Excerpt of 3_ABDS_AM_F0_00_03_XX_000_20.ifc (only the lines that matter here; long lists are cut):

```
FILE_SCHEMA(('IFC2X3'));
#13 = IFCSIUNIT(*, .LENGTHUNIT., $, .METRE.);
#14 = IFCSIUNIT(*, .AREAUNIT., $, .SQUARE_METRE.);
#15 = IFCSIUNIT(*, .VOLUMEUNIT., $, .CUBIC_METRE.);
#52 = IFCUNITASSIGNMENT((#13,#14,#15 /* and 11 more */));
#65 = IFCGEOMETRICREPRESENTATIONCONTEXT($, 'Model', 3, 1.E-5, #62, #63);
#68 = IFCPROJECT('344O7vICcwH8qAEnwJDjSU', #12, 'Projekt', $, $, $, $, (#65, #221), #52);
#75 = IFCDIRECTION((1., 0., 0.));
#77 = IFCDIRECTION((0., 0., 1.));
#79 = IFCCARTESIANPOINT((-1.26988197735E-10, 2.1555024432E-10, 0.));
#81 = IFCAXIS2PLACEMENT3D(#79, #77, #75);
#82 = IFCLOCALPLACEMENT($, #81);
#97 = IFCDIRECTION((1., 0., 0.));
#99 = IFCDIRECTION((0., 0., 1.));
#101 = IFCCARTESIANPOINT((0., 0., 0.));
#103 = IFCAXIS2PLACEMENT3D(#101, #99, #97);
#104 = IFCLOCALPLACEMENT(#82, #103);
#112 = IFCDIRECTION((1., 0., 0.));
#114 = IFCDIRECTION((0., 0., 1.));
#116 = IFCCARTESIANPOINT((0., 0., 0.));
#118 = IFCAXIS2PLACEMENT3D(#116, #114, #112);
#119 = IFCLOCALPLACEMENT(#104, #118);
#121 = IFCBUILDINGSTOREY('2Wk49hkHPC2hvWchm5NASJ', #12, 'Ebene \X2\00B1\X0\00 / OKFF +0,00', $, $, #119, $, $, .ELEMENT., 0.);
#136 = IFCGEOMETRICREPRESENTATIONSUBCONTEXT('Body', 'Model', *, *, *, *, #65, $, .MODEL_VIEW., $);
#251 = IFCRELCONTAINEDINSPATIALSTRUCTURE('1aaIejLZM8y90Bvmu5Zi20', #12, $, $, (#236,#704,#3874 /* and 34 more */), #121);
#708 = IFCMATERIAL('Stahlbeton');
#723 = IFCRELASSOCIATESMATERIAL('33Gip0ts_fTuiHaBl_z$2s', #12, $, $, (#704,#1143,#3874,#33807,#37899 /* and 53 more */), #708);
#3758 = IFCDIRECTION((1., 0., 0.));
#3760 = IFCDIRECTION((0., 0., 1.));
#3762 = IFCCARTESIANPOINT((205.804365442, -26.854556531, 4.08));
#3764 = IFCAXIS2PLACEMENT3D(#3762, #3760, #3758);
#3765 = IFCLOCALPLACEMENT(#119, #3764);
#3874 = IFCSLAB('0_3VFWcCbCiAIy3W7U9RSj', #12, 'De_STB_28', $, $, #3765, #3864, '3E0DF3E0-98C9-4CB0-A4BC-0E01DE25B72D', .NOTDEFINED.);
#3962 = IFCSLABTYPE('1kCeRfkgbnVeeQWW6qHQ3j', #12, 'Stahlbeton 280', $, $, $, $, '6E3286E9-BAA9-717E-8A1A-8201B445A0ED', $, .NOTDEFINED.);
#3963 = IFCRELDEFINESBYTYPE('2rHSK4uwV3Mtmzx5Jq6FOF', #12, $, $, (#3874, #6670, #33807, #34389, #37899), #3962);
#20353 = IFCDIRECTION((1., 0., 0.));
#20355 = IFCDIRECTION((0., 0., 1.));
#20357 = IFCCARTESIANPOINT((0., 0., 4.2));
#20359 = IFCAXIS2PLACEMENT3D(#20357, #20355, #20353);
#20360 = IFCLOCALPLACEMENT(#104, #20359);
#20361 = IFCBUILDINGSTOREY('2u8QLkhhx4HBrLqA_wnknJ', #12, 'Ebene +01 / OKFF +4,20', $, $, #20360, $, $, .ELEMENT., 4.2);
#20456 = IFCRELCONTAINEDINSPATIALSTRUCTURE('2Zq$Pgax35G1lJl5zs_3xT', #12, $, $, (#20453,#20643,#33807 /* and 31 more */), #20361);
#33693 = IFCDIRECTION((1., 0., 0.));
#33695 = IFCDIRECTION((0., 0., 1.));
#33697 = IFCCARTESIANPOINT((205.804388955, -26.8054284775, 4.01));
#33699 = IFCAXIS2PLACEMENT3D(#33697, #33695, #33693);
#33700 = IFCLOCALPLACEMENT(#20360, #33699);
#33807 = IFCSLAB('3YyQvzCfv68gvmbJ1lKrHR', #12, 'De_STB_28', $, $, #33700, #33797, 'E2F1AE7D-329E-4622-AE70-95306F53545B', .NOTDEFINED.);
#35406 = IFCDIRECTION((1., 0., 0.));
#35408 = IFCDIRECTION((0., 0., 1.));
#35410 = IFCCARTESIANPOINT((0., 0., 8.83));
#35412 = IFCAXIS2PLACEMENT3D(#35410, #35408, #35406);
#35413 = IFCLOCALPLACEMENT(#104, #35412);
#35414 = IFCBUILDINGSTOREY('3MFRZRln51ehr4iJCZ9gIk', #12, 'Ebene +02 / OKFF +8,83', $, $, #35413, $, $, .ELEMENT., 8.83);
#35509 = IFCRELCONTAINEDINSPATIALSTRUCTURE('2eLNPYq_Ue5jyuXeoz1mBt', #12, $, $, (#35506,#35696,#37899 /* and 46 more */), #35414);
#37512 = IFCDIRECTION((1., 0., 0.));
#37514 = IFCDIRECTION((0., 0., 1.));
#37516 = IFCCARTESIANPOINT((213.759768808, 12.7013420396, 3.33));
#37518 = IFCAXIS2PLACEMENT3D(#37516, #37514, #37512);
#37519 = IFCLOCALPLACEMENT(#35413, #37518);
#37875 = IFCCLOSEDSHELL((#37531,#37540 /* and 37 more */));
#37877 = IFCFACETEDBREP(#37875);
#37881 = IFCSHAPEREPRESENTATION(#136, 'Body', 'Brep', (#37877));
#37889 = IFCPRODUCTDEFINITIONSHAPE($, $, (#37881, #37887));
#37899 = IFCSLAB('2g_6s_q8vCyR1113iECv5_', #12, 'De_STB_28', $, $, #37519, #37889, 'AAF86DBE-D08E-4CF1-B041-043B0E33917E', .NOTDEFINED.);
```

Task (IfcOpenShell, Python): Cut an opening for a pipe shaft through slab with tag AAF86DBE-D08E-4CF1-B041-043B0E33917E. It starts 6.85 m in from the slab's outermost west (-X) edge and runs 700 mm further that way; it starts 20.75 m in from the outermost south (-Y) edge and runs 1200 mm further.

```python
import numpy as np
import ifcopenshell
import ifcopenshell.api.feature
import ifcopenshell.api.geometry
import ifcopenshell.api.root
import ifcopenshell.geom
import ifcopenshell.util.placement
import ifcopenshell.util.representation
import ifcopenshell.util.shape
import ifcopenshell.util.unit

model = ifcopenshell.open("3_ABDS_AM_F0_00_03_XX_000_20.ifc")
unit_scale = ifcopenshell.util.unit.calculate_unit_scale(model)
settings = ifcopenshell.geom.settings()


def volume(element):
    """Net volume in cubic metres, openings subtracted."""
    shape = ifcopenshell.geom.create_shape(settings, element)
    return ifcopenshell.util.shape.get_volume(shape.geometry)


slab = model.by_guid("2g_6s_q8vCyR1113iECv5_")
before = volume(slab)

# Extent in the slab's own axes, in metres. The edges named are its -X and -Y sides.
slab_shape = ifcopenshell.geom.create_shape(settings, slab)
vertices = ifcopenshell.util.shape.get_vertices(slab_shape.geometry)
x_min, y_min, bottom = vertices.min(axis=0)
top = vertices[:, 2].max()

opening = ifcopenshell.api.root.create_entity(model, ifc_class="IfcOpeningElement", name="Pipe shaft opening")
context = ifcopenshell.util.representation.get_context(model, "Model", "Body", "MODEL_VIEW")
width, depth = 0.7, 1.2
outline = [(0.0, 0.0), (width, 0.0), (width, depth), (0.0, depth), (0.0, 0.0)]
# Overshoot both faces by 50 mm so the cut is clean.
shape = ifcopenshell.api.geometry.add_slab_representation(
    model, context=context, depth=top - bottom + 0.1, polyline=outline
)
ifcopenshell.api.geometry.assign_representation(model, product=opening, representation=shape)

matrix = ifcopenshell.util.placement.get_local_placement(slab.ObjectPlacement)
matrix[:, 3] = matrix @ np.append(np.array([x_min + 6.85, y_min + 20.75, bottom - 0.05]) / unit_scale, 1.0)
ifcopenshell.api.geometry.edit_object_placement(model, product=opening, matrix=matrix, is_si=False)
ifcopenshell.api.feature.add_feature(model, feature=opening, element=slab)

after = volume(slab)

print(f"slab volume {before:.3f} -> {after:.3f} m3")

model.write("3_ABDS_AM_F0_00_03_XX_000_20_rev.ifc")
```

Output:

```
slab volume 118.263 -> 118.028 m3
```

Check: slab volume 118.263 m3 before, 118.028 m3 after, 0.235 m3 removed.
